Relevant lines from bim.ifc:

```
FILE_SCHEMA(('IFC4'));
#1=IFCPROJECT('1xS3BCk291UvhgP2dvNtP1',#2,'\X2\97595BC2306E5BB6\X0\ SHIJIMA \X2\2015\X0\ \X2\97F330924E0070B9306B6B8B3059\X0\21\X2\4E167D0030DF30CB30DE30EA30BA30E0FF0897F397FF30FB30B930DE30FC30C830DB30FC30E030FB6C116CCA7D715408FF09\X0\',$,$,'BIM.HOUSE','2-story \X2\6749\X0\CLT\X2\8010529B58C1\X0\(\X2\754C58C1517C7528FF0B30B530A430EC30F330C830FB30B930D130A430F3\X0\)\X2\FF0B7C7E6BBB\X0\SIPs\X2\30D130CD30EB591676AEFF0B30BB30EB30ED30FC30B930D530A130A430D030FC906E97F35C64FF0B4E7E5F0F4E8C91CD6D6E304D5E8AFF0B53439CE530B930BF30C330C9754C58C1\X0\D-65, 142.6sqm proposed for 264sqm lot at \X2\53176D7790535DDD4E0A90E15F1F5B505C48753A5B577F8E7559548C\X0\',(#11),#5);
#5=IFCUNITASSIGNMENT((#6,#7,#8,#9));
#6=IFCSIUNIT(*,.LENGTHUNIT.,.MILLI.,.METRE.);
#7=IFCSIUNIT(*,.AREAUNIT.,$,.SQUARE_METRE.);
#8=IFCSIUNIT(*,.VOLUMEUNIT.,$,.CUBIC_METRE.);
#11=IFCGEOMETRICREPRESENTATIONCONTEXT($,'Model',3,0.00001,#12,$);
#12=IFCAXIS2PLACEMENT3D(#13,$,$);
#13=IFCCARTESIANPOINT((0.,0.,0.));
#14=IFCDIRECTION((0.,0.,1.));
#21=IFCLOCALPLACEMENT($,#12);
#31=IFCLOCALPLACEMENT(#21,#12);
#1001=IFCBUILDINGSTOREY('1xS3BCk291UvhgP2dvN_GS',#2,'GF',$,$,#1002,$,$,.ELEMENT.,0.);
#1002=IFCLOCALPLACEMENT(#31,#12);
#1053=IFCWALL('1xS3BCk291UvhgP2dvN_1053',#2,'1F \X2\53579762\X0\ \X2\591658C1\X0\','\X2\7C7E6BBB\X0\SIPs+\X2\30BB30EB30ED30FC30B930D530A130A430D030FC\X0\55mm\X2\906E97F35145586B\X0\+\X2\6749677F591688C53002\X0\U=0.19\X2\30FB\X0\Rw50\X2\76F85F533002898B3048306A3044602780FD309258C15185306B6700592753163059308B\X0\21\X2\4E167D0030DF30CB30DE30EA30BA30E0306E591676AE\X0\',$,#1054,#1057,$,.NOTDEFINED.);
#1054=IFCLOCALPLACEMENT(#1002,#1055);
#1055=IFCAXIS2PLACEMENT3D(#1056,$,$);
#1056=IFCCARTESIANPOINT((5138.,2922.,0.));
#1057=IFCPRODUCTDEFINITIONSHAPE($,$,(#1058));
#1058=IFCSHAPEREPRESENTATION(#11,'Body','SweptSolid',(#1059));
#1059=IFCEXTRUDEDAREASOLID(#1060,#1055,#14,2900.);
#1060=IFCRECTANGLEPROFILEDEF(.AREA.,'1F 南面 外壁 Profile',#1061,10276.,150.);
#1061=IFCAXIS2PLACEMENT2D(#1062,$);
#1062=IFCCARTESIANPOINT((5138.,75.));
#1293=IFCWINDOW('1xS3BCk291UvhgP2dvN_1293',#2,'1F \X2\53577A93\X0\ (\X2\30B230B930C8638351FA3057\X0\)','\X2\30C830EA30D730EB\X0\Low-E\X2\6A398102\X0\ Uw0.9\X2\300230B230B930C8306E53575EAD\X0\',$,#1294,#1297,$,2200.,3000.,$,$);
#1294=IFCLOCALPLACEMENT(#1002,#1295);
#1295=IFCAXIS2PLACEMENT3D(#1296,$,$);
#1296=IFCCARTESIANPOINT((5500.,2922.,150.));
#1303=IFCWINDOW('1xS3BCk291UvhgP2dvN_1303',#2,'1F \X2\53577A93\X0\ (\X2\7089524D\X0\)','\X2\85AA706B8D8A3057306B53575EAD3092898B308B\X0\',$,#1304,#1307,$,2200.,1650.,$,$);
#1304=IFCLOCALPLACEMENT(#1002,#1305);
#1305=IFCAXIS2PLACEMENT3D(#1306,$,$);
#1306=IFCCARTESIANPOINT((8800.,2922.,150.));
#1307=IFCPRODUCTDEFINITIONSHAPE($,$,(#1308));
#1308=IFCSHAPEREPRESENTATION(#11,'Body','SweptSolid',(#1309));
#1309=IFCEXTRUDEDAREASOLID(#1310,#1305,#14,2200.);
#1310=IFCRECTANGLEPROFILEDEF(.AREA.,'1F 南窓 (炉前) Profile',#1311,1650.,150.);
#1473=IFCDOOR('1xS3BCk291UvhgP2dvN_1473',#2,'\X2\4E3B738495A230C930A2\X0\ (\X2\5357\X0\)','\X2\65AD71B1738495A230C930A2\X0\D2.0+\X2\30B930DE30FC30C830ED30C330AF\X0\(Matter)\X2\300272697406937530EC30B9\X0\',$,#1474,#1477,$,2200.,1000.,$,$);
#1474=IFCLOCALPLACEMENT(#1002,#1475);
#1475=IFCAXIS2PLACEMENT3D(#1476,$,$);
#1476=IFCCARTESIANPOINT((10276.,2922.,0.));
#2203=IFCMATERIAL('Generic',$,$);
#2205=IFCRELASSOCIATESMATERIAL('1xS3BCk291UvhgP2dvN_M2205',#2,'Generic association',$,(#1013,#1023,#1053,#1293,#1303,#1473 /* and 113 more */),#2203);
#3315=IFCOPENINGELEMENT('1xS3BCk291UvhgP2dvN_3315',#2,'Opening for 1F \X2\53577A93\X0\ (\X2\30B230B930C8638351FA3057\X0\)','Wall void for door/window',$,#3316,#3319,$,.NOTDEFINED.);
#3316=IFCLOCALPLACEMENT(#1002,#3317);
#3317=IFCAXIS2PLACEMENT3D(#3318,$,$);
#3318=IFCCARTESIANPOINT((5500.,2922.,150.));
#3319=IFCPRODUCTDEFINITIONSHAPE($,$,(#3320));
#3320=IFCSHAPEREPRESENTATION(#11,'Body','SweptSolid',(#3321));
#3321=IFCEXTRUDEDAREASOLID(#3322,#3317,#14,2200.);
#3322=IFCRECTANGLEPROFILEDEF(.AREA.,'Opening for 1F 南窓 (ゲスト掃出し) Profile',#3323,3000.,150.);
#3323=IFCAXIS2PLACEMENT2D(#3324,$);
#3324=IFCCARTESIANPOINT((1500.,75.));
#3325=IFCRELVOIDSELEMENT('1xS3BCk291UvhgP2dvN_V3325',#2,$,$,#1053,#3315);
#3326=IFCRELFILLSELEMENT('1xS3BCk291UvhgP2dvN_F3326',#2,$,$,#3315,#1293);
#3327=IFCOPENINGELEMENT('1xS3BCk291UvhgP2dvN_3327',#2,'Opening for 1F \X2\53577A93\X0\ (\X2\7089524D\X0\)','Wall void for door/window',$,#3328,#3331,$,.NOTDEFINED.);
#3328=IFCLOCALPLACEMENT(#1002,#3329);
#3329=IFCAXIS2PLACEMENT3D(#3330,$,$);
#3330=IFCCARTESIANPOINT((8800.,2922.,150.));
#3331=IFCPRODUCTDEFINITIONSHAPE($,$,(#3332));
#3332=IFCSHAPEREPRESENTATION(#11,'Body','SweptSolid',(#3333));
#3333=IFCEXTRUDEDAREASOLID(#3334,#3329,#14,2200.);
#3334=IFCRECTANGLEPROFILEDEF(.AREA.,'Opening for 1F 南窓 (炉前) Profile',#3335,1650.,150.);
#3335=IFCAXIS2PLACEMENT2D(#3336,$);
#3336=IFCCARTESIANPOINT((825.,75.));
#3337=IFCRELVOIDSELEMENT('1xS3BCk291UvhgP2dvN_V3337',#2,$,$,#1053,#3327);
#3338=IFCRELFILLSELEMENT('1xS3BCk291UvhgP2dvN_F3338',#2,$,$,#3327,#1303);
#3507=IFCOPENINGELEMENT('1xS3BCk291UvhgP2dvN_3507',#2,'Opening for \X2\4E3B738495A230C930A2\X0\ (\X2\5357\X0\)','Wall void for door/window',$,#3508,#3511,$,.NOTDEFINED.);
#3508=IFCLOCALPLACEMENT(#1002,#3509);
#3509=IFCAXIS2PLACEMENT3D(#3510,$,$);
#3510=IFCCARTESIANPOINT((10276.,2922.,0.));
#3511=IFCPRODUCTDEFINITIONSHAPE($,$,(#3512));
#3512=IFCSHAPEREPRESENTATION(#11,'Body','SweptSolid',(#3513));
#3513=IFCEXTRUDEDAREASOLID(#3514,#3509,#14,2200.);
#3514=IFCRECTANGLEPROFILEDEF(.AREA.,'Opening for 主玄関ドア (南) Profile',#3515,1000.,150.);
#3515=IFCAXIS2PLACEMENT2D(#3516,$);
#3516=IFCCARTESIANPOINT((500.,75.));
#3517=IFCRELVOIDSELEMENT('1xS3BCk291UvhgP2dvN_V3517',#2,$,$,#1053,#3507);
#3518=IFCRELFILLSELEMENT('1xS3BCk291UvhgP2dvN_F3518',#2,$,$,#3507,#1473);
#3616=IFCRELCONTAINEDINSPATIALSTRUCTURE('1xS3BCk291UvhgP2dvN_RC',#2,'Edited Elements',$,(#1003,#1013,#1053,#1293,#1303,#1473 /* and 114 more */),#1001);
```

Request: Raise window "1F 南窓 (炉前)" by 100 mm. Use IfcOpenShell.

```python
import numpy as np
import ifcopenshell
import ifcopenshell.api.geometry
import ifcopenshell.util.placement
import ifcopenshell.util.unit

model = ifcopenshell.open("bim.ifc")
unit_scale = ifcopenshell.util.unit.calculate_unit_scale(model)

window = model.by_id(1303)
opening = window.FillsVoids[0].RelatingOpeningElement
dz = 0.1 / unit_scale

shift = np.array([0.0, 0.0, dz])
# The window is not placed relative to its opening, so move both.
for product in (opening, window):
    matrix = ifcopenshell.util.placement.get_local_placement(product.ObjectPlacement)
    matrix[:3, 3] += shift
    ifcopenshell.api.geometry.edit_object_placement(model, product=product, matrix=matrix, is_si=False)

print(f"moved by {dz * unit_scale:+.3f} m")

model.write("bim_updated.ifc")
```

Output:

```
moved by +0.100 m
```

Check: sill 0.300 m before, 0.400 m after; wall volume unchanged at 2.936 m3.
